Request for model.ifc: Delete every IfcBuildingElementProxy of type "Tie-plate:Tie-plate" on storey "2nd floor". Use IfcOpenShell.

First a look at what the model holds.

```python
import ifcopenshell
import ifcopenshell.util.element

model = ifcopenshell.open("model.ifc")
print(model.schema)
storey = next(s for s in model.by_type("IfcBuildingStorey") if s.Name == "2nd floor")
proxies = [e for e in ifcopenshell.util.element.get_decomposition(storey) if e.is_a("IfcBuildingElementProxy")]
seen = {}
for e in proxies:
    element_type = ifcopenshell.util.element.get_type(e)
    name = element_type.Name if element_type not in (None, e) else None
    seen[name] = seen.get(name, 0) + 1
for name, count in sorted(seen.items(), key=str):
    print(count, "x", name)
```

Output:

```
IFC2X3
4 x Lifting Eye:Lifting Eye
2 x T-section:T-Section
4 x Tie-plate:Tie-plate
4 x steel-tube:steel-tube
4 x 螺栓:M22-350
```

```python
import ifcopenshell
import ifcopenshell.api.root
import ifcopenshell.util.element

model = ifcopenshell.open("model.ifc")

storey = next(s for s in model.by_type("IfcBuildingStorey") if s.Name == "2nd floor")
proxies = [e for e in ifcopenshell.util.element.get_decomposition(storey) if e.is_a("IfcBuildingElementProxy")]
targets = [e for e in proxies if (t := ifcopenshell.util.element.get_type(e)) not in (None, e) and t.Name == "Tie-plate:Tie-plate"]

for e in targets:
    ifcopenshell.api.root.remove_product(model, product=e)
print(len(targets), "removed")

model.write("model_updated.ifc")
```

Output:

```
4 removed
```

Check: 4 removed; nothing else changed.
